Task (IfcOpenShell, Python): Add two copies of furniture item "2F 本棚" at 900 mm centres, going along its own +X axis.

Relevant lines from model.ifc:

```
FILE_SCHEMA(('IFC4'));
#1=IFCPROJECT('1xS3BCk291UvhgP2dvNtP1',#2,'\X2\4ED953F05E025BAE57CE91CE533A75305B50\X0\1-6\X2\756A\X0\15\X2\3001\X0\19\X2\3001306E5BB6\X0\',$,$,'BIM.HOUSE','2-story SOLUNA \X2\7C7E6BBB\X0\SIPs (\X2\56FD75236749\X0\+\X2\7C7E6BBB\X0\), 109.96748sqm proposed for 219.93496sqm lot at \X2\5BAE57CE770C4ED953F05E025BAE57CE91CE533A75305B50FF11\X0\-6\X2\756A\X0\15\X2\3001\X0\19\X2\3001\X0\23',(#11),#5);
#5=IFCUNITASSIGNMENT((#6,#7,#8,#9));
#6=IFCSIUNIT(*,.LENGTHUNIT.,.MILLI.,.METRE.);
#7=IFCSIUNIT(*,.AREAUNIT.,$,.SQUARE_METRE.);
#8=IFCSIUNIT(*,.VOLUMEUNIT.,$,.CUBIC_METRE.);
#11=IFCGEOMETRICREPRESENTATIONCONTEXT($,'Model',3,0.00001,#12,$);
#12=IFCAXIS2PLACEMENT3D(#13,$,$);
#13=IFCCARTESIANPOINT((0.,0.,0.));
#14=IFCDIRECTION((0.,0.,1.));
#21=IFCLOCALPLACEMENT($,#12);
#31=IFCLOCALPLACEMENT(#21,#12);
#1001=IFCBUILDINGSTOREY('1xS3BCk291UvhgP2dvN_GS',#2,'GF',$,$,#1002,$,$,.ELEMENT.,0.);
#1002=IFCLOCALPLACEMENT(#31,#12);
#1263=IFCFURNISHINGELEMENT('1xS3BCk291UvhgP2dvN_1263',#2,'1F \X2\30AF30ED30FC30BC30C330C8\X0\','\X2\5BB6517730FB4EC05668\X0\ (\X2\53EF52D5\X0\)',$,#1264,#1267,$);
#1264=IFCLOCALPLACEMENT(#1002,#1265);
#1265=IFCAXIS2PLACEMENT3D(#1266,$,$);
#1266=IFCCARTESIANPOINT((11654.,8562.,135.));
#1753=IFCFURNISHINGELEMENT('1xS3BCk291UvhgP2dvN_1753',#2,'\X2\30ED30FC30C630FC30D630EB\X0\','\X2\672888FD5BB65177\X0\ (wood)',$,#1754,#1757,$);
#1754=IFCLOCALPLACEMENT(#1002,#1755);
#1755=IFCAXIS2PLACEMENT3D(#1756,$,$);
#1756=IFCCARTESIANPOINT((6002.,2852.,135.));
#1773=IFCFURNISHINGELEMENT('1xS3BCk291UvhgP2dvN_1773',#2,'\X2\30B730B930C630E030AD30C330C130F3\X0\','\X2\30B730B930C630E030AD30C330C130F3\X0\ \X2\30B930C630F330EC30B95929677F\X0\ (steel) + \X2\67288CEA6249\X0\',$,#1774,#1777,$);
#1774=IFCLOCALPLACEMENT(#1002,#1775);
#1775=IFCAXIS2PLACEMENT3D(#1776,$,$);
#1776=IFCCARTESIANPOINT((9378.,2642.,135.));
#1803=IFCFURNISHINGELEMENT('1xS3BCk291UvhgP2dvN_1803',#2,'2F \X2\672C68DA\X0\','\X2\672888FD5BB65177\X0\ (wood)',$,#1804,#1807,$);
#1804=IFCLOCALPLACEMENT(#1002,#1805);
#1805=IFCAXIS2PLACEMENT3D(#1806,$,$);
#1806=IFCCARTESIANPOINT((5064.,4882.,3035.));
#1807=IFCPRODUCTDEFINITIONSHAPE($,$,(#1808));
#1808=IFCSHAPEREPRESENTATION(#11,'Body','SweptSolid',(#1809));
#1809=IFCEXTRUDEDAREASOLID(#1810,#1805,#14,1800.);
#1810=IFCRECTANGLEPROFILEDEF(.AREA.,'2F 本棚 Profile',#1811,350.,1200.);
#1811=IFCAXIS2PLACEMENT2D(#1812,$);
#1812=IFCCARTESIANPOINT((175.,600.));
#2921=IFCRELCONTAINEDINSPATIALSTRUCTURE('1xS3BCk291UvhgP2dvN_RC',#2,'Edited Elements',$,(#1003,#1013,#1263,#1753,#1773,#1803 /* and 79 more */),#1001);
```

```python
import ifcopenshell
import ifcopenshell.api.geometry
import ifcopenshell.api.root
import ifcopenshell.util.element
import ifcopenshell.util.placement
import ifcopenshell.util.unit

model = ifcopenshell.open("model.ifc")
unit_scale = ifcopenshell.util.unit.calculate_unit_scale(model)


def reuse_history(source, copy):
    """copy_class also copies each property set's owner history, people and application; keep the originals."""
    for rel in copy.IsDefinedBy:
        if rel.is_a("IfcRelDefinesByProperties") and (history := rel.RelatingPropertyDefinition.OwnerHistory):
            rel.RelatingPropertyDefinition.OwnerHistory = source.OwnerHistory
            ifcopenshell.util.element.remove_deep2(model, history)


source = model.by_guid("1xS3BCk291UvhgP2dvN_1803")
base = ifcopenshell.util.placement.get_local_placement(source.ObjectPlacement)
step = base[:3, 0] * 0.9 / unit_scale

for i in range(1, 3):
    copy = ifcopenshell.api.root.copy_class(model, product=source)
    copy.Representation = ifcopenshell.util.element.copy_deep(
        model, source.Representation, exclude=["IfcGeometricRepresentationContext", "IfcRepresentationMap"]
    )
    reuse_history(source, copy)
    matrix = base.copy()
    matrix[:3, 3] += i * step
    print("added at", matrix[:3, 3].round(3) + 0.0)
    ifcopenshell.api.geometry.edit_object_placement(model, product=copy, matrix=matrix, is_si=False)

model.write("model_edited.ifc")
```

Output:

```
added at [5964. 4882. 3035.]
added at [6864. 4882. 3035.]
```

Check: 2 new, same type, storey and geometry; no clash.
